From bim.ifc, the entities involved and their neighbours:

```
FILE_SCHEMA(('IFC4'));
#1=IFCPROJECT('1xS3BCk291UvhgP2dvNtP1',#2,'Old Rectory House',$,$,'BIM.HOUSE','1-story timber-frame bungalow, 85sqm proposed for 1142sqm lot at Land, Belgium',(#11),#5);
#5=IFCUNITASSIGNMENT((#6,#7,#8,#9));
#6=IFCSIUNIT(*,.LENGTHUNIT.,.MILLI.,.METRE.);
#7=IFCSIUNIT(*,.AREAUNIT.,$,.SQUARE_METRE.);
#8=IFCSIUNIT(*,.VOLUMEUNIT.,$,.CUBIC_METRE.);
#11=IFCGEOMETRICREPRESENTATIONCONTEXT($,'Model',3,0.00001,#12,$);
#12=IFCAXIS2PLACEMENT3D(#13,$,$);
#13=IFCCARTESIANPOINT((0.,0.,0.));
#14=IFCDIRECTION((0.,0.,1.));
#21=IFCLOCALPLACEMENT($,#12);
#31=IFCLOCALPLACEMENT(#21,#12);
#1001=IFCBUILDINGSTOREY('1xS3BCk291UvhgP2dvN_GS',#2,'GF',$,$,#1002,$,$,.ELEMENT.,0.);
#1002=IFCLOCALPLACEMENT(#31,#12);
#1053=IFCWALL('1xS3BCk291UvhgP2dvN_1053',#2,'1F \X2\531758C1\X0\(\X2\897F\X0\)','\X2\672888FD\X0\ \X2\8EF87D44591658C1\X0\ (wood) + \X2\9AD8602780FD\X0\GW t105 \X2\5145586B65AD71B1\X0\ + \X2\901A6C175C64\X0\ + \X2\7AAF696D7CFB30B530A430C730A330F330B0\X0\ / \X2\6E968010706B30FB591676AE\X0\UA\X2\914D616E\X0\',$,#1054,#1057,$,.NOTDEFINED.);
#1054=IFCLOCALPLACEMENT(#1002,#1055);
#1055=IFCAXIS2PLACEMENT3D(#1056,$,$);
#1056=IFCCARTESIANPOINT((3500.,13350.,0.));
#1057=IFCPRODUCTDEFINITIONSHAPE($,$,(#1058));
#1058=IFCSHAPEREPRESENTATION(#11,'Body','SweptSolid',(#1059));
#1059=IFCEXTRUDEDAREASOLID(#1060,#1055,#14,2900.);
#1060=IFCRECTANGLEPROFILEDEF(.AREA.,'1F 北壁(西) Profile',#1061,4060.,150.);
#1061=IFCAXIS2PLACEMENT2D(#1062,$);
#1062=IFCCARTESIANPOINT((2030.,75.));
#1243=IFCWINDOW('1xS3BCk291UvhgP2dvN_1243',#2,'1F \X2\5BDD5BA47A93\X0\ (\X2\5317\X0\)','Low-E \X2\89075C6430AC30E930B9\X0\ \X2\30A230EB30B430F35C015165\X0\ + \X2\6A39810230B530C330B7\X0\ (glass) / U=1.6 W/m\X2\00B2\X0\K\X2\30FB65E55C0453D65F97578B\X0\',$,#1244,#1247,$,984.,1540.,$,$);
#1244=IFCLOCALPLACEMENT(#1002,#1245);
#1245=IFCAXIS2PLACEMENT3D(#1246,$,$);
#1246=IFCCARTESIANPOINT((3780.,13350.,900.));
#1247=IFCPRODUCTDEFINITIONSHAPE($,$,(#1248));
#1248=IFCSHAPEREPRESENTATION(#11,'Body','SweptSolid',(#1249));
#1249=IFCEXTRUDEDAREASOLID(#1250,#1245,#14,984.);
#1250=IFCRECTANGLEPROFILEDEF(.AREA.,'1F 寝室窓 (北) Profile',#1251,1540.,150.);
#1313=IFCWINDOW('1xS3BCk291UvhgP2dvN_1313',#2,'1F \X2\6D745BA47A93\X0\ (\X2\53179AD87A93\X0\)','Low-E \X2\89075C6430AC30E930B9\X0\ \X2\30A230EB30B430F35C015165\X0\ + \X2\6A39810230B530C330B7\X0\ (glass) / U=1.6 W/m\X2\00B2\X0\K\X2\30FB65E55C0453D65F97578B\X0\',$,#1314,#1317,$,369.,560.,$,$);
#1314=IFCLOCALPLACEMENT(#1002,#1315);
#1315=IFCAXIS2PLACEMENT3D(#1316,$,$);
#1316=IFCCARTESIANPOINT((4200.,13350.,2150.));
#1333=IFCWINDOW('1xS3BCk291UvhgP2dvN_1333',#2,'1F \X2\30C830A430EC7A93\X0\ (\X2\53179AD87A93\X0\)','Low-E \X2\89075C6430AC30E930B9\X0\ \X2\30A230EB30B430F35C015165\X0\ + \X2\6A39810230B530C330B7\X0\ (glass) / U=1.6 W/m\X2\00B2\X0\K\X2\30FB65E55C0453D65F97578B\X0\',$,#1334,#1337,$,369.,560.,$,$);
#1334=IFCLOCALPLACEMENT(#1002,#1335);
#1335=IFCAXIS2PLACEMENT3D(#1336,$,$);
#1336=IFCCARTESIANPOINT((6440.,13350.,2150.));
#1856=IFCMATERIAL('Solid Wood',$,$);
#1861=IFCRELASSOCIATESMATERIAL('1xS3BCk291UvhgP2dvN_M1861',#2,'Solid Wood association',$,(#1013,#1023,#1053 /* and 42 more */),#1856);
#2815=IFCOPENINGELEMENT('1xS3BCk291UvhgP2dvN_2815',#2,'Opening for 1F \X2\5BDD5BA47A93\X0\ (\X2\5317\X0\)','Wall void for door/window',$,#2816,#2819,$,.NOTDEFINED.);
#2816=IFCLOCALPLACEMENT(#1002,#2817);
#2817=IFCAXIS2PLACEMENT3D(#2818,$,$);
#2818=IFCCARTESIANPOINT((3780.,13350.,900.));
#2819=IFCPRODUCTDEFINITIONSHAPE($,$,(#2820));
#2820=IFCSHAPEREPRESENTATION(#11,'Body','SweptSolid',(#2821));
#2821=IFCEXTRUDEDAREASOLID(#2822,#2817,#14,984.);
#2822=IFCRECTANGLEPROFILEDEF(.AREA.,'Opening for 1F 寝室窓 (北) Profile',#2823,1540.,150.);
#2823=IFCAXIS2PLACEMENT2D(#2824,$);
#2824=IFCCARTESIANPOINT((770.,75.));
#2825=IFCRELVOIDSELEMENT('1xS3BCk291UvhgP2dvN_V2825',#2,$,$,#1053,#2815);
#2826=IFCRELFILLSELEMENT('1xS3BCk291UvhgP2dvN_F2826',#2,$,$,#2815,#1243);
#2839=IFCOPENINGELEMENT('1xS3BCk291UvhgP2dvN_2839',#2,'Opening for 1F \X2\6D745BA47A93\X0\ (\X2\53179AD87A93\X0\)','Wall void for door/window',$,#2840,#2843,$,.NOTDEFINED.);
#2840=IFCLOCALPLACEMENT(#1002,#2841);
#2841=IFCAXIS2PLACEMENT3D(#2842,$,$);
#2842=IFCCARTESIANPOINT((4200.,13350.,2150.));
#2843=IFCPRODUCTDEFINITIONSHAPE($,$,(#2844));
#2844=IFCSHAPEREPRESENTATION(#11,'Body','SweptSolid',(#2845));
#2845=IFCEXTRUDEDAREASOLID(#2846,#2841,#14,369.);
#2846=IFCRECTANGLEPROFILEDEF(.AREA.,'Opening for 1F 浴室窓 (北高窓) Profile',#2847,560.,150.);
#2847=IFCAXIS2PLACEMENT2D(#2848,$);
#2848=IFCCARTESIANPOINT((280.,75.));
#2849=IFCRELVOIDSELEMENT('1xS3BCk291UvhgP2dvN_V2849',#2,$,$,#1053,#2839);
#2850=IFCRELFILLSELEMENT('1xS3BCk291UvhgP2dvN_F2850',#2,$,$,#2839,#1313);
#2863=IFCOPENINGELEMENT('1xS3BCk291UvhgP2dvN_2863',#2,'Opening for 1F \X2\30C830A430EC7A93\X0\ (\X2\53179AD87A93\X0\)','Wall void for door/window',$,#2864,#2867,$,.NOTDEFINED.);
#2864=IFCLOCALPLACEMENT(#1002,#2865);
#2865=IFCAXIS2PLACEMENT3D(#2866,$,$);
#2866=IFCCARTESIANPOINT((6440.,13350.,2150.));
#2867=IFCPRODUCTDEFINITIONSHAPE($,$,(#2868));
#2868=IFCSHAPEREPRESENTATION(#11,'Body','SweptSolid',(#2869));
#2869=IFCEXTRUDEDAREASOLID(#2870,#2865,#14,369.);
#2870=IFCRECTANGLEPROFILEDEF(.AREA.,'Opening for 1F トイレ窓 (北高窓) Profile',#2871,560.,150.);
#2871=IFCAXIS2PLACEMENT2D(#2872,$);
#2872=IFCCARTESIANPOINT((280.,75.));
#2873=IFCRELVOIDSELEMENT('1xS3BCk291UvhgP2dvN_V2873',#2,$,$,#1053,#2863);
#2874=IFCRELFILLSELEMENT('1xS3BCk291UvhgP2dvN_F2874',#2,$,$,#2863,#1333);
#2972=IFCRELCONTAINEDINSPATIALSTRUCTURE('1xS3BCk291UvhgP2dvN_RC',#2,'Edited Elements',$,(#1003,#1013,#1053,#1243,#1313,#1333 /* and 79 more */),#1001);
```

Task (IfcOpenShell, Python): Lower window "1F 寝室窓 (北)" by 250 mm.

```python
import numpy as np
import ifcopenshell
import ifcopenshell.api.geometry
import ifcopenshell.util.placement
import ifcopenshell.util.unit

model = ifcopenshell.open("bim.ifc")
unit_scale = ifcopenshell.util.unit.calculate_unit_scale(model)

window = model.by_guid("1xS3BCk291UvhgP2dvN_1243")
opening = window.FillsVoids[0].RelatingOpeningElement
dz = -250.0

shift = np.array([0.0, 0.0, dz])
# The window is not placed relative to its opening, so move both.
for product in (opening, window):
    matrix = ifcopenshell.util.placement.get_local_placement(product.ObjectPlacement)
    matrix[:3, 3] += shift
    ifcopenshell.api.geometry.edit_object_placement(model, product=product, matrix=matrix, is_si=False)

print(f"moved by {dz * unit_scale:+.3f} m")

model.write("bim_rev.ifc")
```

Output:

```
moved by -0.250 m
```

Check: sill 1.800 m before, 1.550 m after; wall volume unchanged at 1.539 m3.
